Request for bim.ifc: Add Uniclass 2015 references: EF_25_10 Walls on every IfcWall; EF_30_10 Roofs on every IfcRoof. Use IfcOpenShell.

First a look at what the model holds.

```python
import ifcopenshell

model = ifcopenshell.open("bim.ifc")
print(model.schema)
print("classifications:", [c.Name for c in model.by_type("IfcClassification")])
for ifc_class in ("IfcDoor", "IfcRoof", "IfcStair", "IfcWall", "IfcWindow"):
    print(ifc_class, len(model.by_type(ifc_class)))
```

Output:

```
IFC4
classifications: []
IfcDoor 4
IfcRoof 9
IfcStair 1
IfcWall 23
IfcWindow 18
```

```python
import ifcopenshell
import ifcopenshell.api.classification

model = ifcopenshell.open("bim.ifc")

system = ifcopenshell.api.classification.add_classification(model, classification="Uniclass 2015")

codes = {
    "IfcWall": ("EF_25_10", "Walls"),
    "IfcRoof": ("EF_30_10", "Roofs"),
}
for ifc_class, (code, name) in codes.items():
    products = model.by_type(ifc_class)
    ifcopenshell.api.classification.add_reference(
        model, products=products, classification=system, identification=code, name=name
    )
    print(code, len(products))

model.write("bim_v2.ifc")
```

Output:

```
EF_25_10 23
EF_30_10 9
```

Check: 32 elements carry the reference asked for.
